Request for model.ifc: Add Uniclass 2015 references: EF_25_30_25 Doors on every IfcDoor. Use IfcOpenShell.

First a look at what the model holds.

```python
import ifcopenshell

model = ifcopenshell.open("model.ifc")
print(model.schema)
print("classifications:", [c.Name for c in model.by_type("IfcClassification")])
for ifc_class in ("IfcDoor", "IfcRoof", "IfcStair", "IfcWall", "IfcWindow"):
    print(ifc_class, len(model.by_type(ifc_class)))
```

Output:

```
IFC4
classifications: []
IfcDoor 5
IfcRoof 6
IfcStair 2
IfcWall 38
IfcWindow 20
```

```python
import ifcopenshell
import ifcopenshell.api.classification

model = ifcopenshell.open("model.ifc")

system = ifcopenshell.api.classification.add_classification(model, classification="Uniclass 2015")

codes = {
    "IfcDoor": ("EF_25_30_25", "Doors"),
}
for ifc_class, (code, name) in codes.items():
    products = model.by_type(ifc_class)
    ifcopenshell.api.classification.add_reference(
        model, products=products, classification=system, identification=code, name=name
    )
    print(code, len(products))

model.write("model-out.ifc")
```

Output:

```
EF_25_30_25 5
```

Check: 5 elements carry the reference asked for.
